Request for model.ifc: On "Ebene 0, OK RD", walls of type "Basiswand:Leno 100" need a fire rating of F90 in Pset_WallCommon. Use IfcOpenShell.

First a look at what the model holds.

```python
import ifcopenshell
import ifcopenshell.util.element

model = ifcopenshell.open("model.ifc")
print(model.schema)
storey = next(s for s in model.by_type("IfcBuildingStorey") if s.Name == "Ebene 0, OK RD")
walls = [e for e in ifcopenshell.util.element.get_decomposition(storey) if e.is_a("IfcWall")]
seen = {}
for e in walls:
    element_type = ifcopenshell.util.element.get_type(e)
    key = (element_type.Name if element_type != e and element_type else None, ifcopenshell.util.element.get_pset(e, "Pset_WallCommon", "FireRating"))
    seen[key] = seen.get(key, 0) + 1
for (name, value), count in sorted(seen.items(), key=str):
    print(count, "x", name, "|", value)
```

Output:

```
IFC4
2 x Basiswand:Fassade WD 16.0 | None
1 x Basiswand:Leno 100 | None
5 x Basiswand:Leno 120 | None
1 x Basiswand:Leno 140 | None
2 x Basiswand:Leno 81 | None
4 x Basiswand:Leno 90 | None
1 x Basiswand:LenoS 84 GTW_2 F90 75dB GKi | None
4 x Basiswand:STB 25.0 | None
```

```python
import ifcopenshell
import ifcopenshell.api.pset
import ifcopenshell.util.element

model = ifcopenshell.open("model.ifc")

storey = next(s for s in model.by_type("IfcBuildingStorey") if s.Name == "Ebene 0, OK RD")
walls = [e for e in ifcopenshell.util.element.get_decomposition(storey) if e.is_a("IfcWall")]

count = 0
for e in walls:
    element_type = ifcopenshell.util.element.get_type(e)
    if element_type in (None, e) or element_type.Name != "Basiswand:Leno 100":
        continue
    # add_pset returns the element's existing set when there is one.
    pset = ifcopenshell.api.pset.add_pset(model, product=e, name="Pset_WallCommon")
    ifcopenshell.api.pset.edit_pset(model, pset=pset, properties={"FireRating": "F90"})
    count += 1

print(count, "walls updated")

model.write("model_v2.ifc")
```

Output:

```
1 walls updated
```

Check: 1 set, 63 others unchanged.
